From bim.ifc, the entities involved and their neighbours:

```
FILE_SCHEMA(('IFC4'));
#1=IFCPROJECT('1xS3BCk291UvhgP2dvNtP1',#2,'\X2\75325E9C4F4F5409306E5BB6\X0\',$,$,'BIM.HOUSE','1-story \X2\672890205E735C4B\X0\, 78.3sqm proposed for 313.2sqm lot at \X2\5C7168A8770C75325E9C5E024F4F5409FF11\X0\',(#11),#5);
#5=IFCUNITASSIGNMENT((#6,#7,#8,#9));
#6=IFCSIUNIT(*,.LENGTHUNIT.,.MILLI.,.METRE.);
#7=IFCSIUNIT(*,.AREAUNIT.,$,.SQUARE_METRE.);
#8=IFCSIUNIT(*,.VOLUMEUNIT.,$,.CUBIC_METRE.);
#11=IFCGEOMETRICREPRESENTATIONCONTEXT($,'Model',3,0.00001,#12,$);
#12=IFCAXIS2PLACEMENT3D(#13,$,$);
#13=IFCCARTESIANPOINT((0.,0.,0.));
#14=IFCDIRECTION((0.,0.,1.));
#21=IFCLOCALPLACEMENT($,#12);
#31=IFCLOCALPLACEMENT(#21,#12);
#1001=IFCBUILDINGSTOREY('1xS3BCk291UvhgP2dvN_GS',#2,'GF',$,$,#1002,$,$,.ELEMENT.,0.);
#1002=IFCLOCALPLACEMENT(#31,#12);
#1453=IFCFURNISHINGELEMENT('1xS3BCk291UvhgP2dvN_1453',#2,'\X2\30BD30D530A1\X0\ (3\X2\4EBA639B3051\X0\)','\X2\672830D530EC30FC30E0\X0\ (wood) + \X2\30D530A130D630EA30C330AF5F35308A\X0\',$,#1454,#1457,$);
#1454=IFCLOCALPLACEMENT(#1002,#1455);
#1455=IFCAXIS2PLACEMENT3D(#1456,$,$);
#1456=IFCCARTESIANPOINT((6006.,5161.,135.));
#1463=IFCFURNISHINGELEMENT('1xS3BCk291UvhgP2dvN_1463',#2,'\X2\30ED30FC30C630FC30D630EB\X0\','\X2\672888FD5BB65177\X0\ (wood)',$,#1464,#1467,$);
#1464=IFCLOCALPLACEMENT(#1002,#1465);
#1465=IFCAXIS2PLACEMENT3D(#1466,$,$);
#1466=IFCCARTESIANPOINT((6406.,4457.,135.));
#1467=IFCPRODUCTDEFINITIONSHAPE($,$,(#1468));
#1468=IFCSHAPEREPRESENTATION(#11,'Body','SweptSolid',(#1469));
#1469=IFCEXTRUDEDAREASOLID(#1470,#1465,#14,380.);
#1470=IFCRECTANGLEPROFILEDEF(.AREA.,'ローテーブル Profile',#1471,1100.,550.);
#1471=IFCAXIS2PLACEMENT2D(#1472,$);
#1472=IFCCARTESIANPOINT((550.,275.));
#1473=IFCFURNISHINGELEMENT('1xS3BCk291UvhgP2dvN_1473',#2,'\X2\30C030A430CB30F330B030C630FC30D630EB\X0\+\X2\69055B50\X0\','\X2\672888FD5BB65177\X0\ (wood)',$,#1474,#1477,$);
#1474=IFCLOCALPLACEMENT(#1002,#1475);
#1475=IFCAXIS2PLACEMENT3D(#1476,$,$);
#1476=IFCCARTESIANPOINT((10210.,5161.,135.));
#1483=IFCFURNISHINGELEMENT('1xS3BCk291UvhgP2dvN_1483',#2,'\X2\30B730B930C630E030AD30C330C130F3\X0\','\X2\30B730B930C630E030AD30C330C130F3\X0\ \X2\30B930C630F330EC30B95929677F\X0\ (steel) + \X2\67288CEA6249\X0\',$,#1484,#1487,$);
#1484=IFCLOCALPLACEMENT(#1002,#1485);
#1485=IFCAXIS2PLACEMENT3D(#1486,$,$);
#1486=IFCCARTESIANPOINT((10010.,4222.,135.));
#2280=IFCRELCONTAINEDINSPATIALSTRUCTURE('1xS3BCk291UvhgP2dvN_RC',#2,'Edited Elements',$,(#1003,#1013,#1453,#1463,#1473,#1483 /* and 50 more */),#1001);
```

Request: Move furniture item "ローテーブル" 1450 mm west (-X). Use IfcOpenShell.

```python
import ifcopenshell
import ifcopenshell.api.geometry
import ifcopenshell.util.placement
import ifcopenshell.util.unit

model = ifcopenshell.open("bim.ifc")
unit_scale = ifcopenshell.util.unit.calculate_unit_scale(model)

item = model.by_guid("1xS3BCk291UvhgP2dvN_1463")
matrix = ifcopenshell.util.placement.get_local_placement(item.ObjectPlacement)
matrix[0, 3] -= 1.45 / unit_scale
ifcopenshell.api.geometry.edit_object_placement(model, product=item, matrix=matrix, is_si=False)

print(ifcopenshell.util.placement.get_local_placement(item.ObjectPlacement).round(3) + 0.0)

model.write("bim-out.ifc")
```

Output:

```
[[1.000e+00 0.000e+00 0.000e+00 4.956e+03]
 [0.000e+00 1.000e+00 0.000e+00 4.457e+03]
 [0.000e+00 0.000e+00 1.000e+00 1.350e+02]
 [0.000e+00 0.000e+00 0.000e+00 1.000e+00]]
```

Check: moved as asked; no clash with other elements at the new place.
